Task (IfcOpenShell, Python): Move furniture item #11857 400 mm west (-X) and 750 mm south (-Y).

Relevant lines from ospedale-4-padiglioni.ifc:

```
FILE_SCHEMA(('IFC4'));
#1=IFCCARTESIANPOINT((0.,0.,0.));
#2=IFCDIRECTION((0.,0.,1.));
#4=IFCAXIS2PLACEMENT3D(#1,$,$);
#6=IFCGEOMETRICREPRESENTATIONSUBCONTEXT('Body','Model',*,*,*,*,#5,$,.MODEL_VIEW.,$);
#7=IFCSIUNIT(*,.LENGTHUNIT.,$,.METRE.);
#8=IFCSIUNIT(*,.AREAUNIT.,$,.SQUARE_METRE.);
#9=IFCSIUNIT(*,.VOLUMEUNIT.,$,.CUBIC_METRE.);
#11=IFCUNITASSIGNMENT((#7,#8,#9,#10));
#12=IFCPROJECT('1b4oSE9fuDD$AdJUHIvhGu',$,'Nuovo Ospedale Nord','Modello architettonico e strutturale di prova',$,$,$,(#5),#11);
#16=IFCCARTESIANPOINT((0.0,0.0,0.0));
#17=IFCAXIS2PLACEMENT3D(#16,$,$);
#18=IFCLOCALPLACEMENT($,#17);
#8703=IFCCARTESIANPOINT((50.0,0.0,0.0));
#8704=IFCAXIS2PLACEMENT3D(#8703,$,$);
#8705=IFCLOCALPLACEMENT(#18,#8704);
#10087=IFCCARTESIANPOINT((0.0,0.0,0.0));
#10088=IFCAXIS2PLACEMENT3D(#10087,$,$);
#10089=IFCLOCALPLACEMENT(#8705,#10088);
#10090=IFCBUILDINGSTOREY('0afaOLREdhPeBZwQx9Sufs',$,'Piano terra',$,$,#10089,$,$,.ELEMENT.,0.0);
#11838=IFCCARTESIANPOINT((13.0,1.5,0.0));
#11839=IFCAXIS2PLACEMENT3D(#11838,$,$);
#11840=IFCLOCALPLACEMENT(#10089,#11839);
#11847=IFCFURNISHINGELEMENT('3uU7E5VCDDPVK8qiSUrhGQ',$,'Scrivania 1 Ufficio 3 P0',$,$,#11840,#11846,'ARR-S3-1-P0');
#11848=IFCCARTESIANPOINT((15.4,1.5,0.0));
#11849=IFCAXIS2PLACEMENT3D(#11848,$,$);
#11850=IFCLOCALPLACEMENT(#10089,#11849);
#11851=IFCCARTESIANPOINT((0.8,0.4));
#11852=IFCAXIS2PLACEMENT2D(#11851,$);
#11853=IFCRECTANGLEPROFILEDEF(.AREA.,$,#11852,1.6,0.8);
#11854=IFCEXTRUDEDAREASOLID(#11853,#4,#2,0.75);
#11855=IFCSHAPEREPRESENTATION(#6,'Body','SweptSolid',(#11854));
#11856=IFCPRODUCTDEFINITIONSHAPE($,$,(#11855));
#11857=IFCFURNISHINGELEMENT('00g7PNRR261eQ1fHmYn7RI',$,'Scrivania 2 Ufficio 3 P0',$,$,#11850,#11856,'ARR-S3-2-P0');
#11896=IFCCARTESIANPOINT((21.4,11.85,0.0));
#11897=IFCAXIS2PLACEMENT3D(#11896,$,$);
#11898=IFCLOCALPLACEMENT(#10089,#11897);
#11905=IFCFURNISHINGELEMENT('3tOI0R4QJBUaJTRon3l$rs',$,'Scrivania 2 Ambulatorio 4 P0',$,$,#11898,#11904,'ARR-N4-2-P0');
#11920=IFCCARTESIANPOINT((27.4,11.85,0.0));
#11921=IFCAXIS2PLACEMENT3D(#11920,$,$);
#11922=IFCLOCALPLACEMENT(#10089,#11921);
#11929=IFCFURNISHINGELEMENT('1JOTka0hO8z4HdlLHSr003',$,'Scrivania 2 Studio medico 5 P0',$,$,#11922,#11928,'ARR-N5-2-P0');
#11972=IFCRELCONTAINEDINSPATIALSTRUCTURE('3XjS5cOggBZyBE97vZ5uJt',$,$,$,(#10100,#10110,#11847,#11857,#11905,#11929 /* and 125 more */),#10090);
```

```python
import ifcopenshell
import ifcopenshell.api.geometry
import ifcopenshell.util.placement

model = ifcopenshell.open("ospedale-4-padiglioni.ifc")

item = model.by_guid("00g7PNRR261eQ1fHmYn7RI")
matrix = ifcopenshell.util.placement.get_local_placement(item.ObjectPlacement)
matrix[0, 3] -= 0.4
matrix[1, 3] -= 0.75
ifcopenshell.api.geometry.edit_object_placement(model, product=item, matrix=matrix, is_si=False)

print(ifcopenshell.util.placement.get_local_placement(item.ObjectPlacement).round(3) + 0.0)

model.write("ospedale-4-padiglioni_edited.ifc")
```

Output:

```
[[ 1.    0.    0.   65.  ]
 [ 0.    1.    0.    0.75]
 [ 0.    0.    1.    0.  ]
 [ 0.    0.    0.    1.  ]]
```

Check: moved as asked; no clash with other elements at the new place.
